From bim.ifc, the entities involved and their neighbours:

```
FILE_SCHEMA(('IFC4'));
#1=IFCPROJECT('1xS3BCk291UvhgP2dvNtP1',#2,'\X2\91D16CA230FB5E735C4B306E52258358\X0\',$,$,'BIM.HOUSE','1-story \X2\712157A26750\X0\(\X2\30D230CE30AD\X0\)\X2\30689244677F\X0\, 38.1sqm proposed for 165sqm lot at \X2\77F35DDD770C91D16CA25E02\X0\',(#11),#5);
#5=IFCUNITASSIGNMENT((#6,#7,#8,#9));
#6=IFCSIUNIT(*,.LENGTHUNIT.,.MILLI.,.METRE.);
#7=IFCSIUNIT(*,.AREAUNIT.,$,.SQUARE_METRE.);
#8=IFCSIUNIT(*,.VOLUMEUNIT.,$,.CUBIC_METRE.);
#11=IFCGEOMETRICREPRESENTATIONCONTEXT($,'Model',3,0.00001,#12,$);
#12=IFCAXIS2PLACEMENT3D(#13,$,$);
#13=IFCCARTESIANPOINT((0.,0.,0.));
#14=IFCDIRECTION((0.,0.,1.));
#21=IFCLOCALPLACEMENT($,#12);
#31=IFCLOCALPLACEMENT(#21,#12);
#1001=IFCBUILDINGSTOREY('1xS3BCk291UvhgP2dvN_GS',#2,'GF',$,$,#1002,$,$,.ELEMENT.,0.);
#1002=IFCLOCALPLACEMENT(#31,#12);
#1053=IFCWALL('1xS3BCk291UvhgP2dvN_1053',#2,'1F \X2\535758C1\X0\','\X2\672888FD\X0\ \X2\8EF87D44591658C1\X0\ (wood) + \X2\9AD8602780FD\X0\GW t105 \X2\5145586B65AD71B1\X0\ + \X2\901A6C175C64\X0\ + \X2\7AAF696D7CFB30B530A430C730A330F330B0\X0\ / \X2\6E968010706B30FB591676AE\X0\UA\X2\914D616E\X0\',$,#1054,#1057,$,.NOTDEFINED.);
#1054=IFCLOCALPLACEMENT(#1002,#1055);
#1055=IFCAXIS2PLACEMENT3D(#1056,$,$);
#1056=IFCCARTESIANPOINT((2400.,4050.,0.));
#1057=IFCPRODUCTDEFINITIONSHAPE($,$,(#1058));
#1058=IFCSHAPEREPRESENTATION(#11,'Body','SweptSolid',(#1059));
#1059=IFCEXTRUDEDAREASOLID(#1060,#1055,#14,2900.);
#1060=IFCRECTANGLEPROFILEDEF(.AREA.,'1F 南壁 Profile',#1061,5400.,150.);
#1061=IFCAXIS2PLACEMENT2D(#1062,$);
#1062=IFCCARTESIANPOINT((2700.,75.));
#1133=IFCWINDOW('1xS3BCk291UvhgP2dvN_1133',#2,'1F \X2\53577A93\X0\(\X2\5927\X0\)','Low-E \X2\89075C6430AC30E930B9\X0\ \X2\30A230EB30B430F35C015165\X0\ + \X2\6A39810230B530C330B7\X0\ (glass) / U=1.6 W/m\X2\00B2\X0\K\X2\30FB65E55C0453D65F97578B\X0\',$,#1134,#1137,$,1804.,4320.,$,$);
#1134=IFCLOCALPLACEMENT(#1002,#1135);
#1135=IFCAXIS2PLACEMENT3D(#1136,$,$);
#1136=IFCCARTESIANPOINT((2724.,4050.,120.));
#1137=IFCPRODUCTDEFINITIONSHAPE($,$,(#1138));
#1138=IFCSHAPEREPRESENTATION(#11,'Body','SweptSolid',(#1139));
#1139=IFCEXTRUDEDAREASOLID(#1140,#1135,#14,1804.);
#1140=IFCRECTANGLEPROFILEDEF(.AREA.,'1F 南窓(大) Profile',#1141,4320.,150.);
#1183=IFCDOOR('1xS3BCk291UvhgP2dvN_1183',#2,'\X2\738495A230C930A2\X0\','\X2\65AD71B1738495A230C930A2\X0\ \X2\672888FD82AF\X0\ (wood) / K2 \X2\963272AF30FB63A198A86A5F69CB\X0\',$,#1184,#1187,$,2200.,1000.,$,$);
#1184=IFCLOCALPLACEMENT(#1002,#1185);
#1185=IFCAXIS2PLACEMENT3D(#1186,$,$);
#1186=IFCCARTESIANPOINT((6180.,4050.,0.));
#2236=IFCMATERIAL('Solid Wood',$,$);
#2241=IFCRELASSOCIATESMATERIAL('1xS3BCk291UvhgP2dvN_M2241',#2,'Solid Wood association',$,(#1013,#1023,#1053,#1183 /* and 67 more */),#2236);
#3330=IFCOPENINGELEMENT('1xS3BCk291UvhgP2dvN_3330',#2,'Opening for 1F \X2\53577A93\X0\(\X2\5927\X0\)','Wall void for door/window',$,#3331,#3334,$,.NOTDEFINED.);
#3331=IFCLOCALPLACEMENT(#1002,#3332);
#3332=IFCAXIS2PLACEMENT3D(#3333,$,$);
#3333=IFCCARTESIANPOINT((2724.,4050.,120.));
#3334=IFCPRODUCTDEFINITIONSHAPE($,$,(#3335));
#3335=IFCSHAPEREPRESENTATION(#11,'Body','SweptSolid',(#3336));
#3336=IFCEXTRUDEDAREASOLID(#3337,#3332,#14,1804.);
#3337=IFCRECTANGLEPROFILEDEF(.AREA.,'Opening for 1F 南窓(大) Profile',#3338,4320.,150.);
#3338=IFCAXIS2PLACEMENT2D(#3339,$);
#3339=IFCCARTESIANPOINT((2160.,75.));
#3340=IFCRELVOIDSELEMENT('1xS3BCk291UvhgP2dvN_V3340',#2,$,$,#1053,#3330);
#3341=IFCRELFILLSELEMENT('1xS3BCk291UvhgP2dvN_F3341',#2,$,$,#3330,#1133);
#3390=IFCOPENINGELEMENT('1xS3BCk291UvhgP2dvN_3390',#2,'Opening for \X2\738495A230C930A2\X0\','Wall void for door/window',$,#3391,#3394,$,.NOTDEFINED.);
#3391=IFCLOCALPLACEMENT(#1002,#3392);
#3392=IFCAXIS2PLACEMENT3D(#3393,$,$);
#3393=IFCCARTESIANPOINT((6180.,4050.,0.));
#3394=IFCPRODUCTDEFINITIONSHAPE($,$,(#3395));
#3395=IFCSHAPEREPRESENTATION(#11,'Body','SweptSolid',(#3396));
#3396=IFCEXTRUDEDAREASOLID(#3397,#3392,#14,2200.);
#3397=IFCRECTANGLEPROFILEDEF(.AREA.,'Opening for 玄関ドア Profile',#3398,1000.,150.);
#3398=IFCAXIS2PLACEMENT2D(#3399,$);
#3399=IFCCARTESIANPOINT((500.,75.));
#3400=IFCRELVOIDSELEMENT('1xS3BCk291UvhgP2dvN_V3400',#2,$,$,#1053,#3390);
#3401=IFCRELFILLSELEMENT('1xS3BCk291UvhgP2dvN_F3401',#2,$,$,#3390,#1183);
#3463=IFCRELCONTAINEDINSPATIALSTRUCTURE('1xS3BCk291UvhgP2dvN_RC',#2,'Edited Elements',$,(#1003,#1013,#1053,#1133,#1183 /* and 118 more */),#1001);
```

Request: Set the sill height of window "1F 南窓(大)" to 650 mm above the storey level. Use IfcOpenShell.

```python
import numpy as np
import ifcopenshell
import ifcopenshell.api.geometry
import ifcopenshell.geom
import ifcopenshell.util.element
import ifcopenshell.util.placement
import ifcopenshell.util.shape
import ifcopenshell.util.unit

model = ifcopenshell.open("bim.ifc")
unit_scale = ifcopenshell.util.unit.calculate_unit_scale(model)

window = model.by_guid("1xS3BCk291UvhgP2dvN_1133")
opening = window.FillsVoids[0].RelatingOpeningElement
storey = ifcopenshell.util.element.get_container(window, ifc_class="IfcBuildingStorey")
level = ifcopenshell.util.placement.get_local_placement(storey.ObjectPlacement)[2, 3]

# The opening's origin need not be at the sill, so measure its lowest point.
shape = ifcopenshell.geom.create_shape(ifcopenshell.geom.settings(), opening)
bottom = ifcopenshell.util.shape.get_shape_bottom_elevation(shape, shape.geometry) / unit_scale
dz = level + 650.0 - bottom

shift = np.array([0.0, 0.0, dz])
# The window is not placed relative to its opening, so move both.
for product in (opening, window):
    matrix = ifcopenshell.util.placement.get_local_placement(product.ObjectPlacement)
    matrix[:3, 3] += shift
    ifcopenshell.api.geometry.edit_object_placement(model, product=product, matrix=matrix, is_si=False)

print(f"moved by {dz * unit_scale:+.3f} m")

model.write("bim_updated.ifc")
```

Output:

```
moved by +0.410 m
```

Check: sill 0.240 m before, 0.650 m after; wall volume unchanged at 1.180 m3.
